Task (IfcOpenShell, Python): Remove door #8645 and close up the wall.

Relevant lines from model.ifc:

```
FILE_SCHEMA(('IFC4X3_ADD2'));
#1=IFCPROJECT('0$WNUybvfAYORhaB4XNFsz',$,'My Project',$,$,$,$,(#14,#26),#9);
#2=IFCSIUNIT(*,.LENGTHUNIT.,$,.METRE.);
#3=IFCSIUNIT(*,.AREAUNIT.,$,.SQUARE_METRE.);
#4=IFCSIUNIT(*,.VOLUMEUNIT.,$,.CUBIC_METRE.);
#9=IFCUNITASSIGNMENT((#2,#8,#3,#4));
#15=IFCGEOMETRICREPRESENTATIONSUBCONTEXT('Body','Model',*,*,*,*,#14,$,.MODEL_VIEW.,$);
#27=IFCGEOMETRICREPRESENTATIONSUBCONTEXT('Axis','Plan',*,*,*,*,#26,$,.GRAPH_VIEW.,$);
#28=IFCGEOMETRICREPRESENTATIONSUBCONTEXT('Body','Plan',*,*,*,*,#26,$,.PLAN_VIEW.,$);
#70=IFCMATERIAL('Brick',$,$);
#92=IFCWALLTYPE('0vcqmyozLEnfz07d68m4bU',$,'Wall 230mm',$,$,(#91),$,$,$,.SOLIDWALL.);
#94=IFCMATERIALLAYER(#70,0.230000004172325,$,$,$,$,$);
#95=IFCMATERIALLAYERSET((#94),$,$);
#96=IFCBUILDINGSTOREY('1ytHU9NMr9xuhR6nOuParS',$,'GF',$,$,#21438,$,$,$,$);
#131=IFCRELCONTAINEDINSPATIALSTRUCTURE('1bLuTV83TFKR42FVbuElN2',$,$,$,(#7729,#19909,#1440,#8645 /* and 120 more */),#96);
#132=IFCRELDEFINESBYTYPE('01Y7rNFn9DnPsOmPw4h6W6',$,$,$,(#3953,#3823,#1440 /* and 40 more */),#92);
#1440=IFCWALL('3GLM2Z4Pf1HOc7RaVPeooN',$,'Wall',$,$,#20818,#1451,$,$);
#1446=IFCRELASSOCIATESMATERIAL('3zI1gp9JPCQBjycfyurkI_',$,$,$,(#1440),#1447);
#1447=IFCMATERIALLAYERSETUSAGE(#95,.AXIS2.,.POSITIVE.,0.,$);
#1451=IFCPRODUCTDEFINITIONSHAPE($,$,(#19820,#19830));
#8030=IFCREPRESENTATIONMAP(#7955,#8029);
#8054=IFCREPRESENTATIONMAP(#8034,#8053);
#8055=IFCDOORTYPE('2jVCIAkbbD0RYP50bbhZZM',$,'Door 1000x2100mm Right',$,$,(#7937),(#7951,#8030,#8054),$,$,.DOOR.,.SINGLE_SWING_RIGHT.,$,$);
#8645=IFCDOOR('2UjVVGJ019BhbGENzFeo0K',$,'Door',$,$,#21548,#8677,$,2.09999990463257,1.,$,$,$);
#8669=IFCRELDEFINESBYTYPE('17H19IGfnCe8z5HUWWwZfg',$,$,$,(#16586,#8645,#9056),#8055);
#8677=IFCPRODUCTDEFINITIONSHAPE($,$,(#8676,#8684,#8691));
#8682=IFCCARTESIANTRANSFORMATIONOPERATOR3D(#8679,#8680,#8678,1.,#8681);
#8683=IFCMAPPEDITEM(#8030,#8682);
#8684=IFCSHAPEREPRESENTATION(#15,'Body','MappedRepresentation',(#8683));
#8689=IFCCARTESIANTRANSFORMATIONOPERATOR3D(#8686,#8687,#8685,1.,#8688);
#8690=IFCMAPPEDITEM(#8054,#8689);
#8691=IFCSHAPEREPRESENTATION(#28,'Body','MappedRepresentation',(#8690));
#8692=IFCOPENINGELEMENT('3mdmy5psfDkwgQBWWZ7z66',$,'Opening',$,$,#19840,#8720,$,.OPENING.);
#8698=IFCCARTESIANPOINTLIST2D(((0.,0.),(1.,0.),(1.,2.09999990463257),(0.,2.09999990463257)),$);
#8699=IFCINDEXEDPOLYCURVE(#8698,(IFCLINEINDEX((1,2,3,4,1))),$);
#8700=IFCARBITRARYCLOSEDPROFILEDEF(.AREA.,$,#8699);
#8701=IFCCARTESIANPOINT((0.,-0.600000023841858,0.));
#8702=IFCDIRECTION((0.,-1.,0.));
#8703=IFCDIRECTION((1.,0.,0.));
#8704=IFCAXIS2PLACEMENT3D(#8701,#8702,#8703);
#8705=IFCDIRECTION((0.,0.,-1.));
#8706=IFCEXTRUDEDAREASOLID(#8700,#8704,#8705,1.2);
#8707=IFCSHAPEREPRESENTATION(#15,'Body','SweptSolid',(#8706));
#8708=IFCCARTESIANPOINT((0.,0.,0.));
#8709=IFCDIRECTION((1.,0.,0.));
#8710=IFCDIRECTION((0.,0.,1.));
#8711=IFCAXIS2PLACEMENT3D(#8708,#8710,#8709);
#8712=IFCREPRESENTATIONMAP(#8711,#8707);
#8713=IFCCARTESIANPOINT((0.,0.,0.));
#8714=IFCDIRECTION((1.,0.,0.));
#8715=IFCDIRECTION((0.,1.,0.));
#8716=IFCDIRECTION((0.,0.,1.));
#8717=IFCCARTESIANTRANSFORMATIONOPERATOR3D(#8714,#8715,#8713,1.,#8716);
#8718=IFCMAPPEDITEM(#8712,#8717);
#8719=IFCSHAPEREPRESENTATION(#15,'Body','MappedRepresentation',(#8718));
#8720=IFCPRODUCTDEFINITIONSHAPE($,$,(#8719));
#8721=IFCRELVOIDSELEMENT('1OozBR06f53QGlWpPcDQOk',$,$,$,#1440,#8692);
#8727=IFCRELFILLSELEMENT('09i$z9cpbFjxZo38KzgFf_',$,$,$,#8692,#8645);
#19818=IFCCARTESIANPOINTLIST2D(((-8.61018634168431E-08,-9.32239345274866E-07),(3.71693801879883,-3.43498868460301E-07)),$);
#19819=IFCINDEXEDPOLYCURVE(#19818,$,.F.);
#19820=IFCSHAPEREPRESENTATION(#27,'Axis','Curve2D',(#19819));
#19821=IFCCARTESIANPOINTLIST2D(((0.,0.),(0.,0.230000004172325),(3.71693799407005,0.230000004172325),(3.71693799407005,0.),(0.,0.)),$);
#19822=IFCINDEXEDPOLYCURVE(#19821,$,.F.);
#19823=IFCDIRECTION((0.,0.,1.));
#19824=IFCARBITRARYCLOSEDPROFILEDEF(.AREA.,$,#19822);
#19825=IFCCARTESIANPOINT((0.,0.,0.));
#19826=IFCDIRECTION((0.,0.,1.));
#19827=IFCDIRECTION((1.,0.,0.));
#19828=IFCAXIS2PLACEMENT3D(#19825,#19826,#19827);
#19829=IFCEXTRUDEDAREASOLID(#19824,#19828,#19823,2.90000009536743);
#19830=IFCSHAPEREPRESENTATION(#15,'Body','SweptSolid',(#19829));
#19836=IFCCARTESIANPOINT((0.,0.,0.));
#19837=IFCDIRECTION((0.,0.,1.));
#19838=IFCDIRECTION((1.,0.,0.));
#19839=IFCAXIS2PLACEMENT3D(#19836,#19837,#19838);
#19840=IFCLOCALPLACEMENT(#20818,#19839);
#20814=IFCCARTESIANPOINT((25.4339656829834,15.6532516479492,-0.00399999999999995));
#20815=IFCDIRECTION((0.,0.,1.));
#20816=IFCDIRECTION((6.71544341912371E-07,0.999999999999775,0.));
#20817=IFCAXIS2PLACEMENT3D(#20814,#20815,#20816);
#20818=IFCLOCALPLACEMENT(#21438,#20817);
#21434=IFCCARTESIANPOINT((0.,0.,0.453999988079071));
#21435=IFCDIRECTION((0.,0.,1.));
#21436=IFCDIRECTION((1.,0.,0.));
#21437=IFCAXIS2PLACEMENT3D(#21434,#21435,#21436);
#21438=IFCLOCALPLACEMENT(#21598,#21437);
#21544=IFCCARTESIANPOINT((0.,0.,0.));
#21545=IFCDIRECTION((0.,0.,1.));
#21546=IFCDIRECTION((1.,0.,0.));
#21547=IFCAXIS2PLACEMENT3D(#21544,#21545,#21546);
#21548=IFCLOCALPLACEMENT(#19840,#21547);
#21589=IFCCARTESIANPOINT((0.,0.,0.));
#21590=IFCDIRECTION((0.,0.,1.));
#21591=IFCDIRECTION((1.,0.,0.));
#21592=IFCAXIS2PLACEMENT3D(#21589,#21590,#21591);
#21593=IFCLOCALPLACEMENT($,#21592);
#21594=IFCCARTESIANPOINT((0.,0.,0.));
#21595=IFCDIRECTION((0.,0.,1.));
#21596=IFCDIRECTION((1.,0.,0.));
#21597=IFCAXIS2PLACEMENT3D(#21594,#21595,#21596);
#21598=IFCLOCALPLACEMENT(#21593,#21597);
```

```python
import ifcopenshell
import ifcopenshell.api.feature
import ifcopenshell.api.root
import ifcopenshell.geom
import ifcopenshell.util.shape

model = ifcopenshell.open("model.ifc")
settings = ifcopenshell.geom.settings()


def volume(element):
    """Net volume in cubic metres, openings subtracted."""
    shape = ifcopenshell.geom.create_shape(settings, element)
    return ifcopenshell.util.shape.get_volume(shape.geometry)


door = model.by_guid("2UjVVGJ019BhbGENzFeo0K")
opening = door.FillsVoids[0].RelatingOpeningElement
wall = opening.VoidsElements[0].RelatingBuildingElement
before = volume(wall)

ifcopenshell.api.root.remove_product(model, product=door)
ifcopenshell.api.feature.remove_feature(model, feature=opening)

after = volume(wall)

print(f"wall volume {before:.3f} -> {after:.3f} m3")

model.write("model_rev.ifc")
```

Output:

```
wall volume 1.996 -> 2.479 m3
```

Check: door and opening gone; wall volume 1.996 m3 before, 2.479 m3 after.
